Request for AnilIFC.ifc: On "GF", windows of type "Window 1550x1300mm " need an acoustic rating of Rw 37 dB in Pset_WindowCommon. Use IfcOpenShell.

First a look at what the model holds.

```python
import ifcopenshell
import ifcopenshell.util.element

model = ifcopenshell.open("AnilIFC.ifc")
print(model.schema)
storey = next(s for s in model.by_type("IfcBuildingStorey") if s.Name == "GF")
windows = [e for e in ifcopenshell.util.element.get_decomposition(storey) if e.is_a("IfcWindow")]
seen = {}
for e in windows:
    element_type = ifcopenshell.util.element.get_type(e)
    key = (element_type.Name if element_type != e and element_type else None, ifcopenshell.util.element.get_pset(e, "Pset_WindowCommon", "AcousticRating"))
    seen[key] = seen.get(key, 0) + 1
for (name, value), count in sorted(seen.items(), key=str):
    print(count, "x", name, "|", value)
```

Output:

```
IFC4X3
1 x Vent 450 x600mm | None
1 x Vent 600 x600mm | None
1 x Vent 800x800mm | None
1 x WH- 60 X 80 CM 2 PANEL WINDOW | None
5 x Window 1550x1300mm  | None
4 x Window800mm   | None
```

```python
import ifcopenshell
import ifcopenshell.api.pset
import ifcopenshell.util.element

model = ifcopenshell.open("AnilIFC.ifc")

storey = next(s for s in model.by_type("IfcBuildingStorey") if s.Name == "GF")
windows = [e for e in ifcopenshell.util.element.get_decomposition(storey) if e.is_a("IfcWindow")]

count = 0
for e in windows:
    element_type = ifcopenshell.util.element.get_type(e)
    if element_type in (None, e) or element_type.Name != "Window 1550x1300mm ":
        continue
    # add_pset returns the element's existing set when there is one.
    pset = ifcopenshell.api.pset.add_pset(model, product=e, name="Pset_WindowCommon")
    ifcopenshell.api.pset.edit_pset(model, pset=pset, properties={"AcousticRating": "Rw 37 dB"})
    count += 1

print(count, "windows updated")

model.write("AnilIFC_edited.ifc")
```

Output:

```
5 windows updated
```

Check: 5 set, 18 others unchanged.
